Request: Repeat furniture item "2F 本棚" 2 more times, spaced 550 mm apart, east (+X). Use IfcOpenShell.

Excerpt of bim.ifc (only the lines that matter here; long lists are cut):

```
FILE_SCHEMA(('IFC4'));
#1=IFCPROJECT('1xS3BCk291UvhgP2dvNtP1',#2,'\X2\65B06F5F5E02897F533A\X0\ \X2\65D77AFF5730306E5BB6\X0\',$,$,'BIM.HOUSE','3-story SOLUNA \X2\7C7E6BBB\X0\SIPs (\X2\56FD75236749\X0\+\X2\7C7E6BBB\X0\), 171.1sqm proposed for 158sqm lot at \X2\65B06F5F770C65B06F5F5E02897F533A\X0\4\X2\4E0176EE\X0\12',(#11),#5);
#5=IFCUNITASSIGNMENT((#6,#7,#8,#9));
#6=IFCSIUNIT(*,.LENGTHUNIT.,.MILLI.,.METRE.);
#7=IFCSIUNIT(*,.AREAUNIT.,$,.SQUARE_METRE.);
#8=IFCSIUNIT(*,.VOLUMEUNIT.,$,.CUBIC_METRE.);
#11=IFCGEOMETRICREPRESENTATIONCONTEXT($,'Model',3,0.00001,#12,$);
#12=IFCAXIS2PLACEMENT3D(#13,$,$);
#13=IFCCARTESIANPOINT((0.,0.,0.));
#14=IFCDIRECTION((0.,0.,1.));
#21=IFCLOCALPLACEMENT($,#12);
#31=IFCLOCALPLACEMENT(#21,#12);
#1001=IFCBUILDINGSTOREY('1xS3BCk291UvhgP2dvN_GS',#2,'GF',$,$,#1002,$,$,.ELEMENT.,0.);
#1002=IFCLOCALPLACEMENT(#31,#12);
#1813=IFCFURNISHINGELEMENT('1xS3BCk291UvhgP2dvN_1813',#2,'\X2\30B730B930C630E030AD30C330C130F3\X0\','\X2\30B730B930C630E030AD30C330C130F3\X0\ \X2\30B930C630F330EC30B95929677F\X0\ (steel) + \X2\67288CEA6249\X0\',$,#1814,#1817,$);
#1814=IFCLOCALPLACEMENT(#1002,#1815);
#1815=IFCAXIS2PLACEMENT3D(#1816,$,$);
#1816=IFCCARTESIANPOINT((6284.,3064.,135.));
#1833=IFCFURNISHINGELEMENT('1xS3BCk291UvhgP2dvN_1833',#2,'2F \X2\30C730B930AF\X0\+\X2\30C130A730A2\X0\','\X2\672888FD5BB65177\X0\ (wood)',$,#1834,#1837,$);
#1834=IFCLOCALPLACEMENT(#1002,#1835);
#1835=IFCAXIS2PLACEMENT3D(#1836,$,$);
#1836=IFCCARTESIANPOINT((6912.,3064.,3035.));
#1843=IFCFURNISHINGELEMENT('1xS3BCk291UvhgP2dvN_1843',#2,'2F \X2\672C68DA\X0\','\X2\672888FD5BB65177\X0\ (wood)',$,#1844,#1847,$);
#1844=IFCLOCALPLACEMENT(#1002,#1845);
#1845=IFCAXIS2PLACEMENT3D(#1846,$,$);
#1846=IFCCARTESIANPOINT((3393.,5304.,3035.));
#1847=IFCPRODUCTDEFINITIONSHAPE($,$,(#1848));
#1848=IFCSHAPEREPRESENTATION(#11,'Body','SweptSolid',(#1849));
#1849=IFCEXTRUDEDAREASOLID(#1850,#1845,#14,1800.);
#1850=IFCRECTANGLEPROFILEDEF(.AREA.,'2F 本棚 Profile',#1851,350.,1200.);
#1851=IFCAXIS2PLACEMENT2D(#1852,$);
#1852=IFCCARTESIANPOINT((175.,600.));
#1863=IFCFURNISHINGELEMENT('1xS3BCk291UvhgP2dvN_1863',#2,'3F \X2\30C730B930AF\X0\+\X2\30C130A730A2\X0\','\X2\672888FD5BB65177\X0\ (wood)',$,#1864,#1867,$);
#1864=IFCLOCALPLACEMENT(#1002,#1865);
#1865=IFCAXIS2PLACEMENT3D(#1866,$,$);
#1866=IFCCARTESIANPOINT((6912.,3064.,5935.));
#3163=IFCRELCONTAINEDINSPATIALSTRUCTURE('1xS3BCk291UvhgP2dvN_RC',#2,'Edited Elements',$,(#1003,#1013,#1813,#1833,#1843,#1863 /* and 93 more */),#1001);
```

```python
import numpy as np
import ifcopenshell
import ifcopenshell.api.geometry
import ifcopenshell.api.root
import ifcopenshell.util.element
import ifcopenshell.util.placement

model = ifcopenshell.open("bim.ifc")


def reuse_history(source, copy):
    """copy_class also copies each property set's owner history, people and application; keep the originals."""
    for rel in copy.IsDefinedBy:
        if rel.is_a("IfcRelDefinesByProperties") and (history := rel.RelatingPropertyDefinition.OwnerHistory):
            rel.RelatingPropertyDefinition.OwnerHistory = source.OwnerHistory
            ifcopenshell.util.element.remove_deep2(model, history)


source = model.by_id(1843)
base = ifcopenshell.util.placement.get_local_placement(source.ObjectPlacement)
step = np.array([1.0, 0.0, 0.0]) * 550.0

for i in range(1, 3):
    copy = ifcopenshell.api.root.copy_class(model, product=source)
    copy.Representation = ifcopenshell.util.element.copy_deep(
        model, source.Representation, exclude=["IfcGeometricRepresentationContext", "IfcRepresentationMap"]
    )
    reuse_history(source, copy)
    matrix = base.copy()
    matrix[:3, 3] += i * step
    print("added at", matrix[:3, 3].round(3) + 0.0)
    ifcopenshell.api.geometry.edit_object_placement(model, product=copy, matrix=matrix, is_si=False)

model.write("bim_v2.ifc")
```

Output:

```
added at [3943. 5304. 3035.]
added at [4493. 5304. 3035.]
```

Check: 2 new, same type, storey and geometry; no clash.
